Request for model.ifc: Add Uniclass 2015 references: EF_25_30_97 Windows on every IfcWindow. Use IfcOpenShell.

First a look at what the model holds.

```python
import ifcopenshell

model = ifcopenshell.open("model.ifc")
print(model.schema)
print("classifications:", [c.Name for c in model.by_type("IfcClassification")])
for ifc_class in ("IfcDoor", "IfcRoof", "IfcStair", "IfcWall", "IfcWindow"):
    print(ifc_class, len(model.by_type(ifc_class)))
```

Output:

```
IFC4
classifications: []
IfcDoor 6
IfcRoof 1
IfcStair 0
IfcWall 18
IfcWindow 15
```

```python
import ifcopenshell
import ifcopenshell.api.classification

model = ifcopenshell.open("model.ifc")

system = ifcopenshell.api.classification.add_classification(model, classification="Uniclass 2015")

codes = {
    "IfcWindow": ("EF_25_30_97", "Windows"),
}
for ifc_class, (code, name) in codes.items():
    products = model.by_type(ifc_class)
    ifcopenshell.api.classification.add_reference(
        model, products=products, classification=system, identification=code, name=name
    )
    print(code, len(products))

model.write("model_rev.ifc")
```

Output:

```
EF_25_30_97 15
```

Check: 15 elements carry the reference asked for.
